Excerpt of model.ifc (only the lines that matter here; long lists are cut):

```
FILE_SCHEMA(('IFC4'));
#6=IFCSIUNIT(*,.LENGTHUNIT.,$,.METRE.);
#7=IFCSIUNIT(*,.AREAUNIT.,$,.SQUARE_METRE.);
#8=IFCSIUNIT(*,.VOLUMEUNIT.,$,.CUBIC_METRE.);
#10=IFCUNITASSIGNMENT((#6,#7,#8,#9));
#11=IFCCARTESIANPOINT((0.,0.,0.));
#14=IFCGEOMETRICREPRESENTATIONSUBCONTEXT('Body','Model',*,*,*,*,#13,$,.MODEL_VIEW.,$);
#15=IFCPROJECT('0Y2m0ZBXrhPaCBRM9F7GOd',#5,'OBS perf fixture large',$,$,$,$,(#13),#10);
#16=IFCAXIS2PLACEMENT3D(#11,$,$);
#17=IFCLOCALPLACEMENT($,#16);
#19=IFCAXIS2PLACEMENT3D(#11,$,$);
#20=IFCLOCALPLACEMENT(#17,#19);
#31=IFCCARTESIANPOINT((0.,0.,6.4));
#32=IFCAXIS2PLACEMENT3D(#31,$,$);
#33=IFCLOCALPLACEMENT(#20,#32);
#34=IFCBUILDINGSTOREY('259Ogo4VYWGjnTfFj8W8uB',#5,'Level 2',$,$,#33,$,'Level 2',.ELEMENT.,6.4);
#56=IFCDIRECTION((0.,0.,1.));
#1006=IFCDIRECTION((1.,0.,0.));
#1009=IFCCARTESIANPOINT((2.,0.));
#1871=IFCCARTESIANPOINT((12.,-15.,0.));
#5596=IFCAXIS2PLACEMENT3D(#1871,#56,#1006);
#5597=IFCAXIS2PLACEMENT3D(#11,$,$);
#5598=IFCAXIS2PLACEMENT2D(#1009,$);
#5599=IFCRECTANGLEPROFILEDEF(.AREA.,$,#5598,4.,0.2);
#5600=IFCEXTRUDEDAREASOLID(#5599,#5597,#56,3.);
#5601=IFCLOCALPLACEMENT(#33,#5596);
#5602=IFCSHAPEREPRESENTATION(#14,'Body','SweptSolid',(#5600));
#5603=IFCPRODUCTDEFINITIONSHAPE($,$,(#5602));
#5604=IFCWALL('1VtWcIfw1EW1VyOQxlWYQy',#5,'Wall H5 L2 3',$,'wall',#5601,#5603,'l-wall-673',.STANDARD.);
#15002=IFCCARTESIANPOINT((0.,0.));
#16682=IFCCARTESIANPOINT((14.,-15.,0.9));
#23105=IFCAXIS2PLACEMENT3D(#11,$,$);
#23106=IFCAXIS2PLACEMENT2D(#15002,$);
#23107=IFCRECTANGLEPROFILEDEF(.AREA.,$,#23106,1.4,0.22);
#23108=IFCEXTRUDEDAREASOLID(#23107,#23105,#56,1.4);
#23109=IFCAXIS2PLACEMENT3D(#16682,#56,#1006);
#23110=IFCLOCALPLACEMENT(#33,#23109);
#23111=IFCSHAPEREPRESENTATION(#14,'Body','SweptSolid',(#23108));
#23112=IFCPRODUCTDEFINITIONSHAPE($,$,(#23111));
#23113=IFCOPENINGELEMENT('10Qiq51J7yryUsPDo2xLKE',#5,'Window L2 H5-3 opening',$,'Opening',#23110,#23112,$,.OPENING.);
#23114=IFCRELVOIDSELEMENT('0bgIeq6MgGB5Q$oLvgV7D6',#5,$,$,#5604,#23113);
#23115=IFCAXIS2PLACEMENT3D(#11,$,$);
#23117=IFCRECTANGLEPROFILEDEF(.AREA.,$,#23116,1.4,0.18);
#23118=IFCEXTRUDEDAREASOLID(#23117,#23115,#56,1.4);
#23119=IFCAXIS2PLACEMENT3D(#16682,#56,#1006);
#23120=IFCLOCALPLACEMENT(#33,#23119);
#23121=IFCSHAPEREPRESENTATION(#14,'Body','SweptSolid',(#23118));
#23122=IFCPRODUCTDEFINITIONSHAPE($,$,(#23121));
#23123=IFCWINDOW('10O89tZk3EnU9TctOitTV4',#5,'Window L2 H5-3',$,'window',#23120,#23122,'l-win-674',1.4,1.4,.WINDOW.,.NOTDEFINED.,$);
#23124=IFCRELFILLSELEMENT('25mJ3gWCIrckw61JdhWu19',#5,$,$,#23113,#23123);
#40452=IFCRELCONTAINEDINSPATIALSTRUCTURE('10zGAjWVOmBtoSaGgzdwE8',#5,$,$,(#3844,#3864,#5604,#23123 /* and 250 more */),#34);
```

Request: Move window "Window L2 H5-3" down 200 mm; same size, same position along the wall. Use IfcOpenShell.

```python
import numpy as np
import ifcopenshell
import ifcopenshell.api.geometry
import ifcopenshell.util.placement
import ifcopenshell.util.unit

model = ifcopenshell.open("model.ifc")
unit_scale = ifcopenshell.util.unit.calculate_unit_scale(model)

window = model.by_id(23123)
opening = window.FillsVoids[0].RelatingOpeningElement
dz = -0.2 / unit_scale

shift = np.array([0.0, 0.0, dz])
# The window is not placed relative to its opening, so move both.
for product in (opening, window):
    matrix = ifcopenshell.util.placement.get_local_placement(product.ObjectPlacement)
    matrix[:3, 3] += shift
    ifcopenshell.api.geometry.edit_object_placement(model, product=product, matrix=matrix, is_si=False)

print(f"moved by {dz * unit_scale:+.3f} m")

model.write("model_rev.ifc")
```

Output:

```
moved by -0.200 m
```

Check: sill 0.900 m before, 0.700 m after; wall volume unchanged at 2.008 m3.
